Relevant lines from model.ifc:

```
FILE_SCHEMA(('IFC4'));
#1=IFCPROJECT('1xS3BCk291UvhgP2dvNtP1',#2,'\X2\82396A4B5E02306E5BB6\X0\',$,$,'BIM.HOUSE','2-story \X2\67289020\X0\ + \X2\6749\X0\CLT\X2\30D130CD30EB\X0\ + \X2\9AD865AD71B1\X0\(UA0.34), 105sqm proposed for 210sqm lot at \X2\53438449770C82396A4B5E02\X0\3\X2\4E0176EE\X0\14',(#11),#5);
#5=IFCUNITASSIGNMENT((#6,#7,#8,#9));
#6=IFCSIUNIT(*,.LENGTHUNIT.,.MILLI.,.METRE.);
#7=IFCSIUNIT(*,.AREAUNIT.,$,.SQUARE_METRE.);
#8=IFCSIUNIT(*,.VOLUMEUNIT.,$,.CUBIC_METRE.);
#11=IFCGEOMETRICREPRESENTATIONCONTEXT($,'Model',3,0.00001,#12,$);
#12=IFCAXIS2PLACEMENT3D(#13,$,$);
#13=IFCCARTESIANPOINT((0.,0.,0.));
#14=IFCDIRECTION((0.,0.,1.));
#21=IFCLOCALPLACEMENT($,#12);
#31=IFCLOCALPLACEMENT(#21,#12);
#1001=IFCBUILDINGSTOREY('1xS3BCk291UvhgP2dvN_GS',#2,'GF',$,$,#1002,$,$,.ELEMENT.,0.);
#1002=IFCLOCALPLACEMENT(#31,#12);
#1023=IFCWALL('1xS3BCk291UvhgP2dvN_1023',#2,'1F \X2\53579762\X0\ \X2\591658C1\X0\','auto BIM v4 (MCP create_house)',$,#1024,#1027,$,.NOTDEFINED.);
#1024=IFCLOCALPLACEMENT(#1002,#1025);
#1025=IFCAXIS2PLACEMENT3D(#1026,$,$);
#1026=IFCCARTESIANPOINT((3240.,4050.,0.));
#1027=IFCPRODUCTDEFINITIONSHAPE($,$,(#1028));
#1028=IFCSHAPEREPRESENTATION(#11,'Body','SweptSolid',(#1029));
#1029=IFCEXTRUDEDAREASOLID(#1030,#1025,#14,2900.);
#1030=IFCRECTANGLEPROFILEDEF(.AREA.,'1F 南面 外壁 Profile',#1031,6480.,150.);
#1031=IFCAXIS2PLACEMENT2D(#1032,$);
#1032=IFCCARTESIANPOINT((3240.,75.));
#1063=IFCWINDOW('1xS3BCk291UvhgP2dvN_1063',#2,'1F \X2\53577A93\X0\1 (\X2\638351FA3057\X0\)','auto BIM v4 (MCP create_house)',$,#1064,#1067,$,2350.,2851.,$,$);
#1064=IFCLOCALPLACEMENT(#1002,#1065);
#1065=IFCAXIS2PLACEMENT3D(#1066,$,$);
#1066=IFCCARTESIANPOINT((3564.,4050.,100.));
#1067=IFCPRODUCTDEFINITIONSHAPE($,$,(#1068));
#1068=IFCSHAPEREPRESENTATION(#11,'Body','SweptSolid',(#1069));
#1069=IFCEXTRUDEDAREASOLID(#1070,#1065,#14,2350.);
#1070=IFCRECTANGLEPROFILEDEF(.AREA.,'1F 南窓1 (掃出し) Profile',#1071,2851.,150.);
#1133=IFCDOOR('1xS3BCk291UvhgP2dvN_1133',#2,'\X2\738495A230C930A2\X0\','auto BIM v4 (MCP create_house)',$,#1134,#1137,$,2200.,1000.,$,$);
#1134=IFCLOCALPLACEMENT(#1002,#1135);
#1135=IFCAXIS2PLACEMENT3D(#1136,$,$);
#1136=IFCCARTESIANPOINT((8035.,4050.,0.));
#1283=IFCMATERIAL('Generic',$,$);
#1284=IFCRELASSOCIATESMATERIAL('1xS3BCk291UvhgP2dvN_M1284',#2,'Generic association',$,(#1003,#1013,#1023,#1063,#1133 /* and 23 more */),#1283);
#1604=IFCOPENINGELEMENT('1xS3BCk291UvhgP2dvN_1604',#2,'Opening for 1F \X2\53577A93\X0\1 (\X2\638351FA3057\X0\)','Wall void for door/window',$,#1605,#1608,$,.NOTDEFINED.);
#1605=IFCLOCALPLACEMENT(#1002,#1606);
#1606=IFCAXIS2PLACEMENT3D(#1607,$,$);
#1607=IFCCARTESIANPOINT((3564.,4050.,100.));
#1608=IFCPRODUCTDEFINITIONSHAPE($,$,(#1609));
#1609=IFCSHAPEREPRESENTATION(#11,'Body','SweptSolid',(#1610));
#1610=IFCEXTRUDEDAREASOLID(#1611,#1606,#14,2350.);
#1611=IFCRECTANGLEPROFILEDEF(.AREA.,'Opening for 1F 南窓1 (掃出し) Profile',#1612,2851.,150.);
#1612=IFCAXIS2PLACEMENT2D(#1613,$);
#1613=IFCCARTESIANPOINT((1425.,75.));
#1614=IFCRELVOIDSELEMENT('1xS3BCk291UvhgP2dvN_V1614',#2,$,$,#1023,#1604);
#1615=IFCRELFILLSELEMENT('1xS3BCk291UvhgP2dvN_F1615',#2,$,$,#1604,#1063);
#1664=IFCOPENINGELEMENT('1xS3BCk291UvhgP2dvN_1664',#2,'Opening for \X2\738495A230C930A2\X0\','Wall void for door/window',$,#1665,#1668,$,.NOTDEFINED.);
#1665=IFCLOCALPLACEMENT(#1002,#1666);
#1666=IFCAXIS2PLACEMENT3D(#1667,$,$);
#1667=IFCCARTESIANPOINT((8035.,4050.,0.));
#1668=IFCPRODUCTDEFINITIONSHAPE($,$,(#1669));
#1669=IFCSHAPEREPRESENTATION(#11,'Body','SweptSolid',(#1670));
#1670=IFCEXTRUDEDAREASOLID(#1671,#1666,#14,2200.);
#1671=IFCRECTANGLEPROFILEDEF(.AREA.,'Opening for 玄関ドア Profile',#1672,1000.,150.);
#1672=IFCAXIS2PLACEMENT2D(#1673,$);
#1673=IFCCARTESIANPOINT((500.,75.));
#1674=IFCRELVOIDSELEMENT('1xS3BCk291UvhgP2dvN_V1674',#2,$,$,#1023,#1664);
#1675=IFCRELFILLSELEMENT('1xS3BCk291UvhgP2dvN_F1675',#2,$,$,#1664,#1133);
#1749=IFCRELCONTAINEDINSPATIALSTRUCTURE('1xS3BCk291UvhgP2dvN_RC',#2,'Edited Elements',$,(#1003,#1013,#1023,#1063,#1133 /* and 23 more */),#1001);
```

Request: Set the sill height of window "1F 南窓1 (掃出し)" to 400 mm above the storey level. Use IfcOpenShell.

```python
import numpy as np
import ifcopenshell
import ifcopenshell.api.geometry
import ifcopenshell.geom
import ifcopenshell.util.element
import ifcopenshell.util.placement
import ifcopenshell.util.shape
import ifcopenshell.util.unit

model = ifcopenshell.open("model.ifc")
unit_scale = ifcopenshell.util.unit.calculate_unit_scale(model)

window = model.by_id(1063)
opening = window.FillsVoids[0].RelatingOpeningElement
storey = ifcopenshell.util.element.get_container(window, ifc_class="IfcBuildingStorey")
level = ifcopenshell.util.placement.get_local_placement(storey.ObjectPlacement)[2, 3]

# The opening's origin need not be at the sill, so measure its lowest point.
shape = ifcopenshell.geom.create_shape(ifcopenshell.geom.settings(), opening)
bottom = ifcopenshell.util.shape.get_shape_bottom_elevation(shape, shape.geometry) / unit_scale
dz = level + 0.4 / unit_scale - bottom

shift = np.array([0.0, 0.0, dz])
# The window is not placed relative to its opening, so move both.
for product in (opening, window):
    matrix = ifcopenshell.util.placement.get_local_placement(product.ObjectPlacement)
    matrix[:3, 3] += shift
    ifcopenshell.api.geometry.edit_object_placement(model, product=product, matrix=matrix, is_si=False)

print(f"moved by {dz * unit_scale:+.3f} m")

model.write("model_edited.ifc")
```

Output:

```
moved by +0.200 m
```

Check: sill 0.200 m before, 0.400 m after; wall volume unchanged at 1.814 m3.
